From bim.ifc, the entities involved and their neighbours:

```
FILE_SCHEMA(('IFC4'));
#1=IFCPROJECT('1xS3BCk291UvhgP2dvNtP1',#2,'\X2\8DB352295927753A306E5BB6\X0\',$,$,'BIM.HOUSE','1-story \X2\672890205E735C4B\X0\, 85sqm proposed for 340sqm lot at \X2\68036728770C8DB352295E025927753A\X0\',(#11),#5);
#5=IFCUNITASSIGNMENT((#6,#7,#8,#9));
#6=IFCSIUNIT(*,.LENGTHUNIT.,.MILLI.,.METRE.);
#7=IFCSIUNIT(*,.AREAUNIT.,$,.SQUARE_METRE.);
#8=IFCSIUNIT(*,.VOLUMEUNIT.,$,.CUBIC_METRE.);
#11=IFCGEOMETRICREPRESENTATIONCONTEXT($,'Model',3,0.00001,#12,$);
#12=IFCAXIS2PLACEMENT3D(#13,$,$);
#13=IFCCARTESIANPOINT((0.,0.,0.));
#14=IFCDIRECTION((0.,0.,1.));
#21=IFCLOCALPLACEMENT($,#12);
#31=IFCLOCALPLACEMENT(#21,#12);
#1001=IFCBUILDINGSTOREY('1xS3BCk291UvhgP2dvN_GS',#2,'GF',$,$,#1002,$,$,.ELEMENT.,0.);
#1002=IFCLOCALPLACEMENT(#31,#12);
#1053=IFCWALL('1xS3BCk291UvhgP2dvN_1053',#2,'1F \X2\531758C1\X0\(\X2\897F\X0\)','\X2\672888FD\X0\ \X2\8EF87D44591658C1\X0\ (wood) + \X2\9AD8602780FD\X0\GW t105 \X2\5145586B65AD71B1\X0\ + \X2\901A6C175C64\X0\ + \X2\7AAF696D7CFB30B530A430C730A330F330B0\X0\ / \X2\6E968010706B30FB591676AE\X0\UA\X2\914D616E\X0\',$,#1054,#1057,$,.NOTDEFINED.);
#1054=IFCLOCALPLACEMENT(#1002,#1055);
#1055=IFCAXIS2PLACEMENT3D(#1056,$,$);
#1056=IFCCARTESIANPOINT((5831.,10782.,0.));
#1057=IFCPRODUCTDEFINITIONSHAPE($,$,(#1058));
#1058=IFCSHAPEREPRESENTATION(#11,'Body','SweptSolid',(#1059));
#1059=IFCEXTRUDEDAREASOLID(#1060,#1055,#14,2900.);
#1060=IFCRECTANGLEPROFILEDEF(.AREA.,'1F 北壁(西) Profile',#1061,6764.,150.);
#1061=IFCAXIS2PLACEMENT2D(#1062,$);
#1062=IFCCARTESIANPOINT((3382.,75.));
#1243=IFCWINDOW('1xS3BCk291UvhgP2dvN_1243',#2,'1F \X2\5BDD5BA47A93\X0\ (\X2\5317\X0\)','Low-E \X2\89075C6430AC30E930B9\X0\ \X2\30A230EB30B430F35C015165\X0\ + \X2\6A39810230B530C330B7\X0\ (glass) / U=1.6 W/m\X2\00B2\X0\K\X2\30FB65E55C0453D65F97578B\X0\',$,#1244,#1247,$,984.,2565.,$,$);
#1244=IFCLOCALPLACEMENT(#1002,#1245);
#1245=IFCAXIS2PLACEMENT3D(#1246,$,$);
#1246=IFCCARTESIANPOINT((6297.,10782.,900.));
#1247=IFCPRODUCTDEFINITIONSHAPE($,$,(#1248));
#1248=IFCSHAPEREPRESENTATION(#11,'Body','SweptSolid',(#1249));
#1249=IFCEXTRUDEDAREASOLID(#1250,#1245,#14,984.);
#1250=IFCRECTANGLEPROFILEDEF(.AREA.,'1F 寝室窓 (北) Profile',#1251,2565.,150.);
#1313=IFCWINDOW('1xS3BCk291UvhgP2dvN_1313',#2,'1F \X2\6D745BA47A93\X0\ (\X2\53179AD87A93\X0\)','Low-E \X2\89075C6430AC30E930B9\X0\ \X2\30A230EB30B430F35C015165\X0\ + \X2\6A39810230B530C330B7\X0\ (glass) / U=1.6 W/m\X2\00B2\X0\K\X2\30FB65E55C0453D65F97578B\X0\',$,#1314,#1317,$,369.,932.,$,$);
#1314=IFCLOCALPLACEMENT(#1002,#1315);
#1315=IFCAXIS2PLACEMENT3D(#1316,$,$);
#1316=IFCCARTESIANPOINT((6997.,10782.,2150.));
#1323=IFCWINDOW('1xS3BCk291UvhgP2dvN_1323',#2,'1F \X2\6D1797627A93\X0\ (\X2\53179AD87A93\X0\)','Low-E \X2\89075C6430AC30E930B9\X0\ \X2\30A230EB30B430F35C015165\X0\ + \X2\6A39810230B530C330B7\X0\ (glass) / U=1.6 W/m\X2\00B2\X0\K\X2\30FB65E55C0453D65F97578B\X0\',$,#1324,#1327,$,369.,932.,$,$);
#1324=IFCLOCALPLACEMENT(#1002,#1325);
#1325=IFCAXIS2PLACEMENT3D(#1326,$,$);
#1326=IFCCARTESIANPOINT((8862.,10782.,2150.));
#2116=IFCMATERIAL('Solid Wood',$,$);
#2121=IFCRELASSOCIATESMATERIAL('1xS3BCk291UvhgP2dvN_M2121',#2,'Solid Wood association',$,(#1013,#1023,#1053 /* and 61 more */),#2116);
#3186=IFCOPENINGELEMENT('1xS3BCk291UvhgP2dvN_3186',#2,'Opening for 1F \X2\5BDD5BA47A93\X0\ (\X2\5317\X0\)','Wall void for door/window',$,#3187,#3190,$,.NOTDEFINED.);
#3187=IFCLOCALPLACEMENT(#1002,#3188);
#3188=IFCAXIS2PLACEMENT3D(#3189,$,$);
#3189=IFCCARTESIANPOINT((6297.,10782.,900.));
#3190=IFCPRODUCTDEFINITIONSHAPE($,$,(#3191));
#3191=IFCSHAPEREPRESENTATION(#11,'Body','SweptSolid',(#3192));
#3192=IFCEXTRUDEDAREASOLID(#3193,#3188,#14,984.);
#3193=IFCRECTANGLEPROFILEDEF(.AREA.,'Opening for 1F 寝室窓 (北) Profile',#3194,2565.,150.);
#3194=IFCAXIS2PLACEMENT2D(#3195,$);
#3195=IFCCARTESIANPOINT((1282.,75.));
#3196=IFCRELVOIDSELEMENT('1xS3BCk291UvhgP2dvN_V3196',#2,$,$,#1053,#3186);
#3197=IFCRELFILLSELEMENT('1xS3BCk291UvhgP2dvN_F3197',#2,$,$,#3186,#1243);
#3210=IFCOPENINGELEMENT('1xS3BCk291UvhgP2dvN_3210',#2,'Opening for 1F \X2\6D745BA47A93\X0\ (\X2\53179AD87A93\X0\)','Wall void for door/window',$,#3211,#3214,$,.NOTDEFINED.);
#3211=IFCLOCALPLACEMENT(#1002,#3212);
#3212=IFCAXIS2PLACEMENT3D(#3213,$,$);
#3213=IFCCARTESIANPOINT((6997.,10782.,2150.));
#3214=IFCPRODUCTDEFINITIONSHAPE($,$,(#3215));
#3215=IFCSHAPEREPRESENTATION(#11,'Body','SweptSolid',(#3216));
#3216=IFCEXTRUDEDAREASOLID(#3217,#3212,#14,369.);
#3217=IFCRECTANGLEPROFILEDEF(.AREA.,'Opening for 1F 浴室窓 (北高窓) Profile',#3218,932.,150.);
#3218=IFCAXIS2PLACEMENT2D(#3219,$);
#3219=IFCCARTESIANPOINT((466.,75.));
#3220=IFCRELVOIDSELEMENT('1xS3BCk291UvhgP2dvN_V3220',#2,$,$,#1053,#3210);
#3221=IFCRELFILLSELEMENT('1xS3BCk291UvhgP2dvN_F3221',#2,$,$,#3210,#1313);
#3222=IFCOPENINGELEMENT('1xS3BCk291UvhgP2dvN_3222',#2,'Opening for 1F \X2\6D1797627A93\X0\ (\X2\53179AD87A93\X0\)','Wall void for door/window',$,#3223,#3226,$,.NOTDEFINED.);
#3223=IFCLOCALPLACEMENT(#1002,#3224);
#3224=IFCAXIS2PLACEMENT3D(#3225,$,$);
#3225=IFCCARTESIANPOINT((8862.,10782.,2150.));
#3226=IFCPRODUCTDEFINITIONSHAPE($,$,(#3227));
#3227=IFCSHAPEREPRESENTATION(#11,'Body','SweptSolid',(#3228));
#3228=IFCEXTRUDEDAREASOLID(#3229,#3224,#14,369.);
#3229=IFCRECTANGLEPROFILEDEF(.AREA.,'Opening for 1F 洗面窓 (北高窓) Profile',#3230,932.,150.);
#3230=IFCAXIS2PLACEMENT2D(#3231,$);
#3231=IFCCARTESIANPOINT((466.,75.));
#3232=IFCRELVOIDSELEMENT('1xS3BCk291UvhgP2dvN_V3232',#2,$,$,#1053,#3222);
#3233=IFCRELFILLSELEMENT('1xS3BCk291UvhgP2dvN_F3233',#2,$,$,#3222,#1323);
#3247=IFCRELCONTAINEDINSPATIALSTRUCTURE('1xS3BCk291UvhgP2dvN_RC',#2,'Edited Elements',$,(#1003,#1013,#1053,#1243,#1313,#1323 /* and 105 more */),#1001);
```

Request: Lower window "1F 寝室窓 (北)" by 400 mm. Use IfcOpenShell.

```python
import numpy as np
import ifcopenshell
import ifcopenshell.api.geometry
import ifcopenshell.util.placement
import ifcopenshell.util.unit

model = ifcopenshell.open("bim.ifc")
unit_scale = ifcopenshell.util.unit.calculate_unit_scale(model)

window = model.by_id(1243)
opening = window.FillsVoids[0].RelatingOpeningElement
dz = -0.4 / unit_scale

shift = np.array([0.0, 0.0, dz])
# The window is not placed relative to its opening, so move both.
for product in (opening, window):
    matrix = ifcopenshell.util.placement.get_local_placement(product.ObjectPlacement)
    matrix[:3, 3] += shift
    ifcopenshell.api.geometry.edit_object_placement(model, product=product, matrix=matrix, is_si=False)

print(f"moved by {dz * unit_scale:+.3f} m")

model.write("bim_updated.ifc")
```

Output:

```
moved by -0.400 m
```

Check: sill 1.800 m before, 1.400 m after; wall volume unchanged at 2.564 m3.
